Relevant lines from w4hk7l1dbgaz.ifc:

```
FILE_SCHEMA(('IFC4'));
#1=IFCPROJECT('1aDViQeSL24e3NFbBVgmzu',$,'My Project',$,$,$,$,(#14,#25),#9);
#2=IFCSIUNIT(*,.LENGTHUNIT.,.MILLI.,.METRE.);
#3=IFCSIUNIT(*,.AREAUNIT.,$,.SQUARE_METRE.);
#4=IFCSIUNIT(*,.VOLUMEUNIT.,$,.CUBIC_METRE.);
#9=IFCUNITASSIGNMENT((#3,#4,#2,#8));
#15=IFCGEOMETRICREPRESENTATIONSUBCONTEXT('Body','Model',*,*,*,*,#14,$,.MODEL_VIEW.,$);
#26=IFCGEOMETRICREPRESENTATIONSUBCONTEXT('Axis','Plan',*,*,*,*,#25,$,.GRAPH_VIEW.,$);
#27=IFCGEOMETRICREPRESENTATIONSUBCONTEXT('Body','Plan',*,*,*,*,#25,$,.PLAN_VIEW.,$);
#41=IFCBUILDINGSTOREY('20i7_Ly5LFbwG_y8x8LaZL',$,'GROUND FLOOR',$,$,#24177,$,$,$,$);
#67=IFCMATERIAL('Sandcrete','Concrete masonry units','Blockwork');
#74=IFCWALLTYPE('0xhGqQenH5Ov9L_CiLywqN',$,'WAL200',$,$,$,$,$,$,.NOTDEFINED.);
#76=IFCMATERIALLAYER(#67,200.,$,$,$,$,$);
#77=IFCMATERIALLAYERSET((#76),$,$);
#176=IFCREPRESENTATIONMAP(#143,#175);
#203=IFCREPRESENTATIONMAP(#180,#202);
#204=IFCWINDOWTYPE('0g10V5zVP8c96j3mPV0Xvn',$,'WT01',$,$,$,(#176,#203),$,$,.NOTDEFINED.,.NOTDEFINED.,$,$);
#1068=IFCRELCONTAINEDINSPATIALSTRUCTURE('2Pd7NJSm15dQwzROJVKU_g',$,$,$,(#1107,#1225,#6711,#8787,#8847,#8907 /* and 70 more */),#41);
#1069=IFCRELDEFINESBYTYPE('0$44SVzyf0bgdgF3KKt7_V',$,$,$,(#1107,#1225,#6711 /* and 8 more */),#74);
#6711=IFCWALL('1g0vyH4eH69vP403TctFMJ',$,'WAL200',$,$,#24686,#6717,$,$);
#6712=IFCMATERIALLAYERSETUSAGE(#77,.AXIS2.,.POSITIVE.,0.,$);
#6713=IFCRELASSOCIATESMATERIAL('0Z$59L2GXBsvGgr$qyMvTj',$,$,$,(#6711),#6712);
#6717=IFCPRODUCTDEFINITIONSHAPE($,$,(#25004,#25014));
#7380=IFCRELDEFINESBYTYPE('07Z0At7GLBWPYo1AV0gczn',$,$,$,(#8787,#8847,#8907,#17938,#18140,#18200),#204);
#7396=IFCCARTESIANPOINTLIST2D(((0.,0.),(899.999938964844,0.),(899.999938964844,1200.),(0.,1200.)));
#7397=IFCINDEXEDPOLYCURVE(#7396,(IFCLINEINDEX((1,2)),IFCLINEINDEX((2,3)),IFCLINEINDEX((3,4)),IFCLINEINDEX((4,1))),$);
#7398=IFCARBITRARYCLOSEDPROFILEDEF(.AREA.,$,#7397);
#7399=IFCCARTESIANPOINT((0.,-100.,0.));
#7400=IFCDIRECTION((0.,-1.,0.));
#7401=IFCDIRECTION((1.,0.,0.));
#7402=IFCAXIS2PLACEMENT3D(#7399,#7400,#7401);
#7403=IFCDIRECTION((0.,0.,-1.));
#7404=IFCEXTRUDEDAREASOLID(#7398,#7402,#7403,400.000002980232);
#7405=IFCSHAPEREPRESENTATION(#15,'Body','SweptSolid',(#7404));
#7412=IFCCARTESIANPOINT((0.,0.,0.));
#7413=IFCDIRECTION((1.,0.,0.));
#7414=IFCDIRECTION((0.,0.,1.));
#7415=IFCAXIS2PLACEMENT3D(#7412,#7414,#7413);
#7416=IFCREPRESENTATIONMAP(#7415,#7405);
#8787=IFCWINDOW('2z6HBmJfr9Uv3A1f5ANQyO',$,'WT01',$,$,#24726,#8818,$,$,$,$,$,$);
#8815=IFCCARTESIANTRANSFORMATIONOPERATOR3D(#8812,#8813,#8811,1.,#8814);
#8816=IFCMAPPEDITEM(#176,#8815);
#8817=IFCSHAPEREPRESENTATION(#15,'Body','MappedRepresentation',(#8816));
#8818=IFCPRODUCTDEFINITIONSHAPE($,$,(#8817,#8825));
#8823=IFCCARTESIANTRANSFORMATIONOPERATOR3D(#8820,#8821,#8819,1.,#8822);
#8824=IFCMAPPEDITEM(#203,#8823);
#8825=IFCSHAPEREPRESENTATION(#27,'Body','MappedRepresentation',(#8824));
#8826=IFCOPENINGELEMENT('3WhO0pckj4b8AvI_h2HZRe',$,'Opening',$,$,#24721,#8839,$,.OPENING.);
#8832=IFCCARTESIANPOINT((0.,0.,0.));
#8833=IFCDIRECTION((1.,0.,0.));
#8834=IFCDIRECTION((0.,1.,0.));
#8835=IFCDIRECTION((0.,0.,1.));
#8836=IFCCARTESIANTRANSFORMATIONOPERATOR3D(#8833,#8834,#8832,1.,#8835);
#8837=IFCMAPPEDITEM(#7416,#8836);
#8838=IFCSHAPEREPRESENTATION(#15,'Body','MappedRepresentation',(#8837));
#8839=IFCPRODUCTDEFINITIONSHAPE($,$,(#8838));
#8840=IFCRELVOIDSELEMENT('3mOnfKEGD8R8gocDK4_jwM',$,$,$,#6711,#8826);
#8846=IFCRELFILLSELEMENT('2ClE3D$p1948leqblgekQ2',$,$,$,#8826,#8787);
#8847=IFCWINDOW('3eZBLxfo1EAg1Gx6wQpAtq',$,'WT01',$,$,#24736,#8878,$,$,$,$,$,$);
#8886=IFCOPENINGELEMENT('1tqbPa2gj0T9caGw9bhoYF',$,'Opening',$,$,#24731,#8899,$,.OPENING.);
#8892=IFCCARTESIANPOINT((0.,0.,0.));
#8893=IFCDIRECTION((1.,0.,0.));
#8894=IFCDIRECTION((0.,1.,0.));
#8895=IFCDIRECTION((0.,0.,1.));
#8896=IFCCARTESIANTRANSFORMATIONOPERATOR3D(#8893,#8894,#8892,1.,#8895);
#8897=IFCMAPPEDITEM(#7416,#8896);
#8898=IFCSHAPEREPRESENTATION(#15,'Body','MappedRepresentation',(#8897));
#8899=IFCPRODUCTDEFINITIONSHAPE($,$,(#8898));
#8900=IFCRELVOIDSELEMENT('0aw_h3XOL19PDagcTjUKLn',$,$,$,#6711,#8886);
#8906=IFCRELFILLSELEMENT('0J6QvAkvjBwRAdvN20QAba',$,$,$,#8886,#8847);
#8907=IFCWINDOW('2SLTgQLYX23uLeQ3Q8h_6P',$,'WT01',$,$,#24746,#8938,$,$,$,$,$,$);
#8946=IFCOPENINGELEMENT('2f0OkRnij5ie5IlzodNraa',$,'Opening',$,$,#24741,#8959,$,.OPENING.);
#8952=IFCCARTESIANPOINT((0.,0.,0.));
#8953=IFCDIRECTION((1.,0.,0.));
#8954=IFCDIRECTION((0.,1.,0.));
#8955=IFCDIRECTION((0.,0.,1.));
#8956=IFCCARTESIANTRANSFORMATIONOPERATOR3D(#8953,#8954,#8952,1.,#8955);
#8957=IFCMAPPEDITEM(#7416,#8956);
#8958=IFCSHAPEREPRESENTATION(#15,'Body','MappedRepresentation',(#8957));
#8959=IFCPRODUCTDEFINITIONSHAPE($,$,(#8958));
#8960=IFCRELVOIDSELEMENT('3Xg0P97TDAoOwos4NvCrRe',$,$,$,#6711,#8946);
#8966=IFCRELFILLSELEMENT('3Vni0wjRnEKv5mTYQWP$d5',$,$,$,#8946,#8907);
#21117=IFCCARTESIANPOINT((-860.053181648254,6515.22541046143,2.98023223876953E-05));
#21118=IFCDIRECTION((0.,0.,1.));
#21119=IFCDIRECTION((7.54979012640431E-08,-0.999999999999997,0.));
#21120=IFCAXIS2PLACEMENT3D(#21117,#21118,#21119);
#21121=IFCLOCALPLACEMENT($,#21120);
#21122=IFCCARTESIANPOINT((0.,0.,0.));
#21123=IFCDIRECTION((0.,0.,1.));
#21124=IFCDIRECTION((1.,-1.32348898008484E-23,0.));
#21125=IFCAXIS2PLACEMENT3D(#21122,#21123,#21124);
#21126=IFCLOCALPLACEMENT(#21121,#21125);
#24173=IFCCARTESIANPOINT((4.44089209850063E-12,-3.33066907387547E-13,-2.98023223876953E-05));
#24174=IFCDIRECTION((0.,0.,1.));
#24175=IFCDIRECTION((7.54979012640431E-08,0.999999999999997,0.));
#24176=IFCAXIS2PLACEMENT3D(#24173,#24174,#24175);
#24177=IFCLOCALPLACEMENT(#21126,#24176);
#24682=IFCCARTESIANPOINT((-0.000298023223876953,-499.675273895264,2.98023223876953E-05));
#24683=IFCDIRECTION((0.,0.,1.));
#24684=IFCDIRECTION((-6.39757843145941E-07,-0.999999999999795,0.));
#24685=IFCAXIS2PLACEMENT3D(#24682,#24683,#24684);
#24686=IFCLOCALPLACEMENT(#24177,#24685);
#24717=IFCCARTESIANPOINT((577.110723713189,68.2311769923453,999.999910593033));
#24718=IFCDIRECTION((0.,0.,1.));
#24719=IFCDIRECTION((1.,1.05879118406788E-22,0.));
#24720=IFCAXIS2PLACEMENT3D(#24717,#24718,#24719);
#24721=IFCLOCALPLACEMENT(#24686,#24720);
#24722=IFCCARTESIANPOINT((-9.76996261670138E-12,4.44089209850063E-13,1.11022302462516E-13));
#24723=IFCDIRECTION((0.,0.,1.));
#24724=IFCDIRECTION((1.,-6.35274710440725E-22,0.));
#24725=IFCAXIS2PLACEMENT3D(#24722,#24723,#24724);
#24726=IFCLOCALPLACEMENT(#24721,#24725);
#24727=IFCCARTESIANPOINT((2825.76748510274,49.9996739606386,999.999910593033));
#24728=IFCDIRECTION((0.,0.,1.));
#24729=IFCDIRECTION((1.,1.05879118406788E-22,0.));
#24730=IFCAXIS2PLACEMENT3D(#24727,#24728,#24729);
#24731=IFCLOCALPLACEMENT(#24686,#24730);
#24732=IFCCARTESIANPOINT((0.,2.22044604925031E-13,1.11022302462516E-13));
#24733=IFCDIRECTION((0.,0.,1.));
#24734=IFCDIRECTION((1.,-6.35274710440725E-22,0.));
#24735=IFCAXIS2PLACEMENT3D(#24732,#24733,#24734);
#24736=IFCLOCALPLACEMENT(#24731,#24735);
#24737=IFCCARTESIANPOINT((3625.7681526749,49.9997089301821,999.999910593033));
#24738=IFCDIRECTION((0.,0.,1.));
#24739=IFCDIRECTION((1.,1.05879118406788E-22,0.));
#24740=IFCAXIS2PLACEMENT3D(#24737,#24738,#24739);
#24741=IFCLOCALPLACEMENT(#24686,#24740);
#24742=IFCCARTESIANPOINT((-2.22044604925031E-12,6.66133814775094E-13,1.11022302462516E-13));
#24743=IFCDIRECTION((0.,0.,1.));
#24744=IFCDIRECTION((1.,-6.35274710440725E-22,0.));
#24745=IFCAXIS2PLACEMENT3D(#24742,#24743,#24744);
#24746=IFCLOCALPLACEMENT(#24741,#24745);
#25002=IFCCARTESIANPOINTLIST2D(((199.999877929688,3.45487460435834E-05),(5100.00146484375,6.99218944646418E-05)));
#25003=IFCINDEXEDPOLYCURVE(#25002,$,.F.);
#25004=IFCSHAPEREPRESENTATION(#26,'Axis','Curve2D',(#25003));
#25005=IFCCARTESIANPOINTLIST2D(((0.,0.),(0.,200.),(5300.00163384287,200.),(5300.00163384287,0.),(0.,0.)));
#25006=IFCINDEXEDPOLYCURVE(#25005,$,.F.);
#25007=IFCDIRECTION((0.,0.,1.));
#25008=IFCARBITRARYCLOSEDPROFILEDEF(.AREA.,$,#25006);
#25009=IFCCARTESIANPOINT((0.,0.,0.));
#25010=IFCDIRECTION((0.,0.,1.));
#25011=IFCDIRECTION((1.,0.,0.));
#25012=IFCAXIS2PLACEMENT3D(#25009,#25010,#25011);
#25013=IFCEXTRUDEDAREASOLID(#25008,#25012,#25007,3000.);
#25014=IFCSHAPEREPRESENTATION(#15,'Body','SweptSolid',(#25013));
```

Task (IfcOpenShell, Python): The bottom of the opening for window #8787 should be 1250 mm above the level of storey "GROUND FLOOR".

```python
import numpy as np
import ifcopenshell
import ifcopenshell.api.geometry
import ifcopenshell.geom
import ifcopenshell.util.element
import ifcopenshell.util.placement
import ifcopenshell.util.shape
import ifcopenshell.util.unit

model = ifcopenshell.open("w4hk7l1dbgaz.ifc")
unit_scale = ifcopenshell.util.unit.calculate_unit_scale(model)

window = model.by_guid("2z6HBmJfr9Uv3A1f5ANQyO")
opening = window.FillsVoids[0].RelatingOpeningElement
storey = ifcopenshell.util.element.get_container(window, ifc_class="IfcBuildingStorey")
level = ifcopenshell.util.placement.get_local_placement(storey.ObjectPlacement)[2, 3]

# The opening's origin need not be at the sill, so measure its lowest point.
shape = ifcopenshell.geom.create_shape(ifcopenshell.geom.settings(), opening)
bottom = ifcopenshell.util.shape.get_shape_bottom_elevation(shape, shape.geometry) / unit_scale
dz = level + 1.25 / unit_scale - bottom

shift = np.array([0.0, 0.0, dz])
# The window is placed relative to its opening, so it follows when the opening moves.
matrix = ifcopenshell.util.placement.get_local_placement(opening.ObjectPlacement)
matrix[:3, 3] += shift
ifcopenshell.api.geometry.edit_object_placement(
    model, product=opening, matrix=matrix, is_si=False, should_transform_children=True
)

print(f"moved by {dz * unit_scale:+.3f} m")

model.write("w4hk7l1dbgaz-out.ifc")
```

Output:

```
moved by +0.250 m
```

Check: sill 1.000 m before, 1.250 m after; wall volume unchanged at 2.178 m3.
